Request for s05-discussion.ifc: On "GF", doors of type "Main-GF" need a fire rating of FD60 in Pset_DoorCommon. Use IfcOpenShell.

First a look at what the model holds.

```python
import ifcopenshell
import ifcopenshell.util.element

model = ifcopenshell.open("s05-discussion.ifc")
print(model.schema)
storey = next(s for s in model.by_type("IfcBuildingStorey") if s.Name == "GF")
doors = [e for e in ifcopenshell.util.element.get_decomposition(storey) if e.is_a("IfcDoor")]
seen = {}
for e in doors:
    element_type = ifcopenshell.util.element.get_type(e)
    key = (element_type.Name if element_type != e and element_type else None, ifcopenshell.util.element.get_pset(e, "Pset_DoorCommon", "FireRating"))
    seen[key] = seen.get(key, 0) + 1
for (name, value), count in sorted(seen.items(), key=str):
    print(count, "x", name, "|", value)
```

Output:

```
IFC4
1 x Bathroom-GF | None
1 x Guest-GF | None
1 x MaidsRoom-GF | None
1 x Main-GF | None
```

```python
import ifcopenshell
import ifcopenshell.api.pset
import ifcopenshell.util.element

model = ifcopenshell.open("s05-discussion.ifc")

storey = next(s for s in model.by_type("IfcBuildingStorey") if s.Name == "GF")
doors = [e for e in ifcopenshell.util.element.get_decomposition(storey) if e.is_a("IfcDoor")]

count = 0
for e in doors:
    element_type = ifcopenshell.util.element.get_type(e)
    if element_type in (None, e) or element_type.Name != "Main-GF":
        continue
    # add_pset returns the element's existing set when there is one.
    pset = ifcopenshell.api.pset.add_pset(model, product=e, name="Pset_DoorCommon")
    ifcopenshell.api.pset.edit_pset(model, pset=pset, properties={"FireRating": "FD60"})
    count += 1

print(count, "doors updated")

model.write("s05-discussion_v2.ifc")
```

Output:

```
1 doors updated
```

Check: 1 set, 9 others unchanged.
